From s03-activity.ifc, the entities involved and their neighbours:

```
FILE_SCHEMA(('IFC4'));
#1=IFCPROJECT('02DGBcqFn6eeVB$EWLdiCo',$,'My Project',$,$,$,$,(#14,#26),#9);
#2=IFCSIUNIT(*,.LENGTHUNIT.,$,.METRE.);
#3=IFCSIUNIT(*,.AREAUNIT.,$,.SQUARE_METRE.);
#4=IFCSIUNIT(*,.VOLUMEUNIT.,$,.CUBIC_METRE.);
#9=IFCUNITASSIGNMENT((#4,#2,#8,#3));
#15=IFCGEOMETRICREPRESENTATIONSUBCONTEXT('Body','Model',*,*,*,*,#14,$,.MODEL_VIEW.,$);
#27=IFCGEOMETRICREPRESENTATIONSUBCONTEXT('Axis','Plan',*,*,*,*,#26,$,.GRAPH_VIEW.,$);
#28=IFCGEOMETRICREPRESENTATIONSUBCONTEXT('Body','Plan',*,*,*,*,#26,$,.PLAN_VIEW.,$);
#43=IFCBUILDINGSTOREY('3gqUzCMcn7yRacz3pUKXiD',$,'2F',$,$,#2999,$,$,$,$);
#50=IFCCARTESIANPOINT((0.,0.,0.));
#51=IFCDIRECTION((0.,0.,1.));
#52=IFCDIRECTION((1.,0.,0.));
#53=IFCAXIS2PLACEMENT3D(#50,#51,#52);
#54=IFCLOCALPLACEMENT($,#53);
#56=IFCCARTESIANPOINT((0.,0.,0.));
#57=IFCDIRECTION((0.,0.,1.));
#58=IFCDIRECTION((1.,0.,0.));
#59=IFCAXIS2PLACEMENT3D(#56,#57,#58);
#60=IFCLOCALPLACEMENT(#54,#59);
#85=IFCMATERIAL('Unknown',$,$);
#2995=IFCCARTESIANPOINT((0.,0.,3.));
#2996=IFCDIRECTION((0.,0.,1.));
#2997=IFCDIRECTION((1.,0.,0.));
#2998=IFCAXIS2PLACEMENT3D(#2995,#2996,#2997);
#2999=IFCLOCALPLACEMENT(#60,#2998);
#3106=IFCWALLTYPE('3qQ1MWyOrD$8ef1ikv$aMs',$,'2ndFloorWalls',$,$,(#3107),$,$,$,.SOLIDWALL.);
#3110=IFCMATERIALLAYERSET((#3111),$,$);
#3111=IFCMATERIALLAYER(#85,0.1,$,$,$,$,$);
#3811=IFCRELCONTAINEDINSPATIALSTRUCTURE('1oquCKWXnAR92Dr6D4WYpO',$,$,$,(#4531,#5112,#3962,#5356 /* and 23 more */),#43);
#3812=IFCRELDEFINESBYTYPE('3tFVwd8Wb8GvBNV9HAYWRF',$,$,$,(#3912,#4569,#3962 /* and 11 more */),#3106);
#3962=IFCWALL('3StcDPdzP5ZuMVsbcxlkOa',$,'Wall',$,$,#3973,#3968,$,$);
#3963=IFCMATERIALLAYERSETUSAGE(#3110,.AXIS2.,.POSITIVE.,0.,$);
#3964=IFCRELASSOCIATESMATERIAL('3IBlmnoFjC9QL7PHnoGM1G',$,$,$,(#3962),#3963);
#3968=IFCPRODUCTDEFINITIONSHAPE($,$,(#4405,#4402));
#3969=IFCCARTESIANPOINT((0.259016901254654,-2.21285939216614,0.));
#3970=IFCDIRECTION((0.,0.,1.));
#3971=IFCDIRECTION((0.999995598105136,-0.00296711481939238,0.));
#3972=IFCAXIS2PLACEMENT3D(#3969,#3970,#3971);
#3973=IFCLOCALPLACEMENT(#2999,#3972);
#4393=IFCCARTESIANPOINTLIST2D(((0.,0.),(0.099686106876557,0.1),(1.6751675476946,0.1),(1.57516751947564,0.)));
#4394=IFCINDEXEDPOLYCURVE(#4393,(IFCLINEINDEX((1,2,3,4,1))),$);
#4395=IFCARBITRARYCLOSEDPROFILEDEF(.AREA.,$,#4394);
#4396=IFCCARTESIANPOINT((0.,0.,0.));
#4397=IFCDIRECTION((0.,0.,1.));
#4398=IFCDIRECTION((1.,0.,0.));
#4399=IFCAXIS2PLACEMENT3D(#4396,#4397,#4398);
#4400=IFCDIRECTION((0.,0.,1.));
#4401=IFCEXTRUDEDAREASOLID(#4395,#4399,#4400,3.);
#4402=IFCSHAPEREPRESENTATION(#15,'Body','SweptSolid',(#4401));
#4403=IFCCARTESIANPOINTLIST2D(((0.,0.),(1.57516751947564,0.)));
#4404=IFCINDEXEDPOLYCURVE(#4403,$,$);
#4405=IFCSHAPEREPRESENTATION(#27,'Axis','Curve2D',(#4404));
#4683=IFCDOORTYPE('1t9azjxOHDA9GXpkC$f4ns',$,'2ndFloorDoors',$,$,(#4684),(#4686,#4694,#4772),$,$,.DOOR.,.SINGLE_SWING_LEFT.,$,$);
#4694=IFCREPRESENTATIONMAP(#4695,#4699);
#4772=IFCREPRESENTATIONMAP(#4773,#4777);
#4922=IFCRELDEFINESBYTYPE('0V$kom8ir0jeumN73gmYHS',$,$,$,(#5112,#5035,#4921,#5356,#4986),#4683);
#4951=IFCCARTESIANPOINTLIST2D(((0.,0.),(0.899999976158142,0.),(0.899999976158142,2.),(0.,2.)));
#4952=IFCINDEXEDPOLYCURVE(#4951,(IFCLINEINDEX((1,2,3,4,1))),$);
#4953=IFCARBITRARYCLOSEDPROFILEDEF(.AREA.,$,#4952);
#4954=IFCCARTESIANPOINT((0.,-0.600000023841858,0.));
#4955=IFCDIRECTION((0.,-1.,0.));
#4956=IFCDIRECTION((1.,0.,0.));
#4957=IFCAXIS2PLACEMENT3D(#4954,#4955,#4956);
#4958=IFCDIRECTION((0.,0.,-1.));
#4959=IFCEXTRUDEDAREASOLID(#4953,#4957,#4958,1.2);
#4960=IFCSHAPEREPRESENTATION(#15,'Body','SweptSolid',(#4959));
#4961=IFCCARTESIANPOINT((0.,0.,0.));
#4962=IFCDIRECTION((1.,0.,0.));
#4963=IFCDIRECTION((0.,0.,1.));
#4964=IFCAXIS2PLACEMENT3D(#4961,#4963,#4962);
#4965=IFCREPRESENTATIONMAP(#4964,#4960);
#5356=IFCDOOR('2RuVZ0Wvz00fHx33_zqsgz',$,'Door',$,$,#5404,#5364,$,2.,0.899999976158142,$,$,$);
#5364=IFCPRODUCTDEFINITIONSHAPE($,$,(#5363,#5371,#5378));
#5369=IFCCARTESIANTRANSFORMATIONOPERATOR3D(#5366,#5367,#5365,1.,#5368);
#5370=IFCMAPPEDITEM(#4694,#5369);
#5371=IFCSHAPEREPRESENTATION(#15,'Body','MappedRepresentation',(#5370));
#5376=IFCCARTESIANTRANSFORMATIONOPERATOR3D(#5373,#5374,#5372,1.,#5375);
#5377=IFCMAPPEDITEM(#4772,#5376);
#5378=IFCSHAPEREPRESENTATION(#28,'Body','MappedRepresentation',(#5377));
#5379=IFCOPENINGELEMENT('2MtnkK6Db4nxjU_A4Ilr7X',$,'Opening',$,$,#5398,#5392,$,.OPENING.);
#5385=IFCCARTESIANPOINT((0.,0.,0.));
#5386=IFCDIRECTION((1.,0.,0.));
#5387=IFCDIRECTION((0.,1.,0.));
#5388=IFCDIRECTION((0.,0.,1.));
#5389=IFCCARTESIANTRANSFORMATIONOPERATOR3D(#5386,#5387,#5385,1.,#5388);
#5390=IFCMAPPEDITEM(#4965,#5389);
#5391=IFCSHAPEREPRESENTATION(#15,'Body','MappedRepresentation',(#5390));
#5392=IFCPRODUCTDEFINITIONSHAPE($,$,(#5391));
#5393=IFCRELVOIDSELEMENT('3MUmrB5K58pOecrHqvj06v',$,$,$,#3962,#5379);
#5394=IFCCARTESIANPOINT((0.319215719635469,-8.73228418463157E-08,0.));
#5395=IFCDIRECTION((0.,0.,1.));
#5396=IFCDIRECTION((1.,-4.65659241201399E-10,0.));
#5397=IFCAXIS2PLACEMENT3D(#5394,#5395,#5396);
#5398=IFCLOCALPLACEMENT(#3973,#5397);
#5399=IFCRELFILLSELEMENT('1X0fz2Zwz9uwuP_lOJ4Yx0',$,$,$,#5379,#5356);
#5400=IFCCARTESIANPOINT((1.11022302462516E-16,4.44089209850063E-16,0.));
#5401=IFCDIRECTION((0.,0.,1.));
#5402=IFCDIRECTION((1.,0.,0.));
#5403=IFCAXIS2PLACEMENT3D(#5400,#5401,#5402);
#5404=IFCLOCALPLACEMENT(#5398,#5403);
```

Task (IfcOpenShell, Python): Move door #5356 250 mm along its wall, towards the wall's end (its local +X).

```python
import ifcopenshell
import ifcopenshell.api.geometry
import ifcopenshell.util.placement

model = ifcopenshell.open("s03-activity.ifc")

door = model.by_guid("2RuVZ0Wvz00fHx33_zqsgz")
opening = door.FillsVoids[0].RelatingOpeningElement
wall = opening.VoidsElements[0].RelatingBuildingElement

wall_matrix = ifcopenshell.util.placement.get_local_placement(wall.ObjectPlacement)
shift = wall_matrix[:3, 0] * 0.25
before = ifcopenshell.util.placement.get_local_placement(door.ObjectPlacement)[:3, 3].copy()

# The door is placed relative to its opening, so it follows when the opening moves.
matrix = ifcopenshell.util.placement.get_local_placement(opening.ObjectPlacement)
matrix[:3, 3] += shift
ifcopenshell.api.geometry.edit_object_placement(
    model, product=opening, matrix=matrix, is_si=False, should_transform_children=True
)

after = ifcopenshell.util.placement.get_local_placement(door.ObjectPlacement)[:3, 3]
print("door moved by", (after - before).round(3) + 0.0)

model.write("s03-activity_v2.ifc")
```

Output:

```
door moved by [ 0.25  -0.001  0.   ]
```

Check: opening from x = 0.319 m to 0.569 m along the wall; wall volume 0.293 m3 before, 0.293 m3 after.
